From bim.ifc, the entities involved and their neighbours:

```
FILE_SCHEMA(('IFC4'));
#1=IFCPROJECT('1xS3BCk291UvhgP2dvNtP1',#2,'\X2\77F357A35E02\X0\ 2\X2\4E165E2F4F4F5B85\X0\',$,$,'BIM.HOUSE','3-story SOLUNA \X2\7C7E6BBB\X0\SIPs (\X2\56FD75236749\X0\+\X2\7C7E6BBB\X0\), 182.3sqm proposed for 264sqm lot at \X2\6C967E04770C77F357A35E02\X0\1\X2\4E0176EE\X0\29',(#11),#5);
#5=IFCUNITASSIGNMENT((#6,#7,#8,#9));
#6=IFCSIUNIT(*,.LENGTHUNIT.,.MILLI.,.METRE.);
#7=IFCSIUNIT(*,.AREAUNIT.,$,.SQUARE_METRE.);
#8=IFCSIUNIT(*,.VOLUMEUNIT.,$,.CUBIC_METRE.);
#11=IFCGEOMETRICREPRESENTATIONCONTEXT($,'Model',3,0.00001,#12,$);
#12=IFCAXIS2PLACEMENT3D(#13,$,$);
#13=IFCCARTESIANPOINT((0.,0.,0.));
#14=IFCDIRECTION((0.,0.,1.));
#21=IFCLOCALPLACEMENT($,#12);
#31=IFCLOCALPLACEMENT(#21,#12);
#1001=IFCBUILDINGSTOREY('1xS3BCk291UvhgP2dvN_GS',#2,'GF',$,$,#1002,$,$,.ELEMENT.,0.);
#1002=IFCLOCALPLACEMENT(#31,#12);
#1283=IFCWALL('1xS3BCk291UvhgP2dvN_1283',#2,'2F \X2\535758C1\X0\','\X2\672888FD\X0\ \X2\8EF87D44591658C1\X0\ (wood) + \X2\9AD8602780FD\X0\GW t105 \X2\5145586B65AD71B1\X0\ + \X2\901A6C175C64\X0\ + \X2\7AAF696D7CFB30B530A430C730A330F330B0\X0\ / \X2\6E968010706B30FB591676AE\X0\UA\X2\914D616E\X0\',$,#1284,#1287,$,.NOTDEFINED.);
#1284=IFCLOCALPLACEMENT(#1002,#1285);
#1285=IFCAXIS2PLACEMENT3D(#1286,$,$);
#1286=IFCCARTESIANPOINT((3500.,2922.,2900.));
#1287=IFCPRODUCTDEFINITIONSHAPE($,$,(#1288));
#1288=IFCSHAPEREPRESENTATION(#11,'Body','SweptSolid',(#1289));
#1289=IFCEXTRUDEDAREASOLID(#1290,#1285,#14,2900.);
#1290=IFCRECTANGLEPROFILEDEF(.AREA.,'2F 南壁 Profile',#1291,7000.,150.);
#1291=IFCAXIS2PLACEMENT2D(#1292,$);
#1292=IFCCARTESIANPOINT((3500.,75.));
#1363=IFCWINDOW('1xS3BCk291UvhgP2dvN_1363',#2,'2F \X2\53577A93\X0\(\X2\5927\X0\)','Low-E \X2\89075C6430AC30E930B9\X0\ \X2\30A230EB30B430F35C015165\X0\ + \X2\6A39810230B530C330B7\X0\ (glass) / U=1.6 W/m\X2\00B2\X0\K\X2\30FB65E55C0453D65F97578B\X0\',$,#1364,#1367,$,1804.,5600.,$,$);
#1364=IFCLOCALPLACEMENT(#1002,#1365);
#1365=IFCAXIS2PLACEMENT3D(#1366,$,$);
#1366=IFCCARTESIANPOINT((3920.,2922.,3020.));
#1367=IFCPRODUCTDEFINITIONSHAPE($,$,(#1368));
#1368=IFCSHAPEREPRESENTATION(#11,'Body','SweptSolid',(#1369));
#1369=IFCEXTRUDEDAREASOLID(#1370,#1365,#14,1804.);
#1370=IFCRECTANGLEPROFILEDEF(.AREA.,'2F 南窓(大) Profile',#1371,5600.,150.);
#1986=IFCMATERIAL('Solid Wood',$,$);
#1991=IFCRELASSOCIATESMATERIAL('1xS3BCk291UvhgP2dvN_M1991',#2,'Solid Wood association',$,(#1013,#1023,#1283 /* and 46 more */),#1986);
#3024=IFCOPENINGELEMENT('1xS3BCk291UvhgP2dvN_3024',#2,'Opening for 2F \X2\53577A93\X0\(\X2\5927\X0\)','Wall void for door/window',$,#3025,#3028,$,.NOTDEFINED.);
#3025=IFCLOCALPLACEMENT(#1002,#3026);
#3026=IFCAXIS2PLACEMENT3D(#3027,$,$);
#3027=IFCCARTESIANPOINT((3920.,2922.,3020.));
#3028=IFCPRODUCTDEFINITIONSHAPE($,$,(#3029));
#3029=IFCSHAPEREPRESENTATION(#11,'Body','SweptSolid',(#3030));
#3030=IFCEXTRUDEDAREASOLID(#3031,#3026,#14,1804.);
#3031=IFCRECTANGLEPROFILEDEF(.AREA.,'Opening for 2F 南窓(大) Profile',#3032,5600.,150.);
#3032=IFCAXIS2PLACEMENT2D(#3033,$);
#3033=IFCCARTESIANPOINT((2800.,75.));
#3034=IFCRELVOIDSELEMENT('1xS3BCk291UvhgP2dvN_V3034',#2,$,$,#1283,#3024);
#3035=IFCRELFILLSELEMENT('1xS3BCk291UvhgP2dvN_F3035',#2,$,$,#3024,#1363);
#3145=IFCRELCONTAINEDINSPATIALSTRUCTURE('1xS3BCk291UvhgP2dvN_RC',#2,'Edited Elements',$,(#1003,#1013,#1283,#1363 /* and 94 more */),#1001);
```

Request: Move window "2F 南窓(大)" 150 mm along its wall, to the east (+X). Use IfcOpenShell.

```python
import ifcopenshell
import ifcopenshell.api.geometry
import ifcopenshell.util.placement
import ifcopenshell.util.unit

model = ifcopenshell.open("bim.ifc")
unit_scale = ifcopenshell.util.unit.calculate_unit_scale(model)

window = model.by_guid("1xS3BCk291UvhgP2dvN_1363")
opening = window.FillsVoids[0].RelatingOpeningElement
wall = opening.VoidsElements[0].RelatingBuildingElement

wall_matrix = ifcopenshell.util.placement.get_local_placement(wall.ObjectPlacement)
shift = wall_matrix[:3, 0] * 0.15 / unit_scale
before = ifcopenshell.util.placement.get_local_placement(window.ObjectPlacement)[:3, 3].copy()

# The window is not placed relative to its opening, so move both.
for product in (opening, window):
    matrix = ifcopenshell.util.placement.get_local_placement(product.ObjectPlacement)
    matrix[:3, 3] += shift
    ifcopenshell.api.geometry.edit_object_placement(model, product=product, matrix=matrix, is_si=False)

after = ifcopenshell.util.placement.get_local_placement(window.ObjectPlacement)[:3, 3]
print("window moved by", (after - before).round(3) + 0.0)

model.write("bim-out.ifc")
```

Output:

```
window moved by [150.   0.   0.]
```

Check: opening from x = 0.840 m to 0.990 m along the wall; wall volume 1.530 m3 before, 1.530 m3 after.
